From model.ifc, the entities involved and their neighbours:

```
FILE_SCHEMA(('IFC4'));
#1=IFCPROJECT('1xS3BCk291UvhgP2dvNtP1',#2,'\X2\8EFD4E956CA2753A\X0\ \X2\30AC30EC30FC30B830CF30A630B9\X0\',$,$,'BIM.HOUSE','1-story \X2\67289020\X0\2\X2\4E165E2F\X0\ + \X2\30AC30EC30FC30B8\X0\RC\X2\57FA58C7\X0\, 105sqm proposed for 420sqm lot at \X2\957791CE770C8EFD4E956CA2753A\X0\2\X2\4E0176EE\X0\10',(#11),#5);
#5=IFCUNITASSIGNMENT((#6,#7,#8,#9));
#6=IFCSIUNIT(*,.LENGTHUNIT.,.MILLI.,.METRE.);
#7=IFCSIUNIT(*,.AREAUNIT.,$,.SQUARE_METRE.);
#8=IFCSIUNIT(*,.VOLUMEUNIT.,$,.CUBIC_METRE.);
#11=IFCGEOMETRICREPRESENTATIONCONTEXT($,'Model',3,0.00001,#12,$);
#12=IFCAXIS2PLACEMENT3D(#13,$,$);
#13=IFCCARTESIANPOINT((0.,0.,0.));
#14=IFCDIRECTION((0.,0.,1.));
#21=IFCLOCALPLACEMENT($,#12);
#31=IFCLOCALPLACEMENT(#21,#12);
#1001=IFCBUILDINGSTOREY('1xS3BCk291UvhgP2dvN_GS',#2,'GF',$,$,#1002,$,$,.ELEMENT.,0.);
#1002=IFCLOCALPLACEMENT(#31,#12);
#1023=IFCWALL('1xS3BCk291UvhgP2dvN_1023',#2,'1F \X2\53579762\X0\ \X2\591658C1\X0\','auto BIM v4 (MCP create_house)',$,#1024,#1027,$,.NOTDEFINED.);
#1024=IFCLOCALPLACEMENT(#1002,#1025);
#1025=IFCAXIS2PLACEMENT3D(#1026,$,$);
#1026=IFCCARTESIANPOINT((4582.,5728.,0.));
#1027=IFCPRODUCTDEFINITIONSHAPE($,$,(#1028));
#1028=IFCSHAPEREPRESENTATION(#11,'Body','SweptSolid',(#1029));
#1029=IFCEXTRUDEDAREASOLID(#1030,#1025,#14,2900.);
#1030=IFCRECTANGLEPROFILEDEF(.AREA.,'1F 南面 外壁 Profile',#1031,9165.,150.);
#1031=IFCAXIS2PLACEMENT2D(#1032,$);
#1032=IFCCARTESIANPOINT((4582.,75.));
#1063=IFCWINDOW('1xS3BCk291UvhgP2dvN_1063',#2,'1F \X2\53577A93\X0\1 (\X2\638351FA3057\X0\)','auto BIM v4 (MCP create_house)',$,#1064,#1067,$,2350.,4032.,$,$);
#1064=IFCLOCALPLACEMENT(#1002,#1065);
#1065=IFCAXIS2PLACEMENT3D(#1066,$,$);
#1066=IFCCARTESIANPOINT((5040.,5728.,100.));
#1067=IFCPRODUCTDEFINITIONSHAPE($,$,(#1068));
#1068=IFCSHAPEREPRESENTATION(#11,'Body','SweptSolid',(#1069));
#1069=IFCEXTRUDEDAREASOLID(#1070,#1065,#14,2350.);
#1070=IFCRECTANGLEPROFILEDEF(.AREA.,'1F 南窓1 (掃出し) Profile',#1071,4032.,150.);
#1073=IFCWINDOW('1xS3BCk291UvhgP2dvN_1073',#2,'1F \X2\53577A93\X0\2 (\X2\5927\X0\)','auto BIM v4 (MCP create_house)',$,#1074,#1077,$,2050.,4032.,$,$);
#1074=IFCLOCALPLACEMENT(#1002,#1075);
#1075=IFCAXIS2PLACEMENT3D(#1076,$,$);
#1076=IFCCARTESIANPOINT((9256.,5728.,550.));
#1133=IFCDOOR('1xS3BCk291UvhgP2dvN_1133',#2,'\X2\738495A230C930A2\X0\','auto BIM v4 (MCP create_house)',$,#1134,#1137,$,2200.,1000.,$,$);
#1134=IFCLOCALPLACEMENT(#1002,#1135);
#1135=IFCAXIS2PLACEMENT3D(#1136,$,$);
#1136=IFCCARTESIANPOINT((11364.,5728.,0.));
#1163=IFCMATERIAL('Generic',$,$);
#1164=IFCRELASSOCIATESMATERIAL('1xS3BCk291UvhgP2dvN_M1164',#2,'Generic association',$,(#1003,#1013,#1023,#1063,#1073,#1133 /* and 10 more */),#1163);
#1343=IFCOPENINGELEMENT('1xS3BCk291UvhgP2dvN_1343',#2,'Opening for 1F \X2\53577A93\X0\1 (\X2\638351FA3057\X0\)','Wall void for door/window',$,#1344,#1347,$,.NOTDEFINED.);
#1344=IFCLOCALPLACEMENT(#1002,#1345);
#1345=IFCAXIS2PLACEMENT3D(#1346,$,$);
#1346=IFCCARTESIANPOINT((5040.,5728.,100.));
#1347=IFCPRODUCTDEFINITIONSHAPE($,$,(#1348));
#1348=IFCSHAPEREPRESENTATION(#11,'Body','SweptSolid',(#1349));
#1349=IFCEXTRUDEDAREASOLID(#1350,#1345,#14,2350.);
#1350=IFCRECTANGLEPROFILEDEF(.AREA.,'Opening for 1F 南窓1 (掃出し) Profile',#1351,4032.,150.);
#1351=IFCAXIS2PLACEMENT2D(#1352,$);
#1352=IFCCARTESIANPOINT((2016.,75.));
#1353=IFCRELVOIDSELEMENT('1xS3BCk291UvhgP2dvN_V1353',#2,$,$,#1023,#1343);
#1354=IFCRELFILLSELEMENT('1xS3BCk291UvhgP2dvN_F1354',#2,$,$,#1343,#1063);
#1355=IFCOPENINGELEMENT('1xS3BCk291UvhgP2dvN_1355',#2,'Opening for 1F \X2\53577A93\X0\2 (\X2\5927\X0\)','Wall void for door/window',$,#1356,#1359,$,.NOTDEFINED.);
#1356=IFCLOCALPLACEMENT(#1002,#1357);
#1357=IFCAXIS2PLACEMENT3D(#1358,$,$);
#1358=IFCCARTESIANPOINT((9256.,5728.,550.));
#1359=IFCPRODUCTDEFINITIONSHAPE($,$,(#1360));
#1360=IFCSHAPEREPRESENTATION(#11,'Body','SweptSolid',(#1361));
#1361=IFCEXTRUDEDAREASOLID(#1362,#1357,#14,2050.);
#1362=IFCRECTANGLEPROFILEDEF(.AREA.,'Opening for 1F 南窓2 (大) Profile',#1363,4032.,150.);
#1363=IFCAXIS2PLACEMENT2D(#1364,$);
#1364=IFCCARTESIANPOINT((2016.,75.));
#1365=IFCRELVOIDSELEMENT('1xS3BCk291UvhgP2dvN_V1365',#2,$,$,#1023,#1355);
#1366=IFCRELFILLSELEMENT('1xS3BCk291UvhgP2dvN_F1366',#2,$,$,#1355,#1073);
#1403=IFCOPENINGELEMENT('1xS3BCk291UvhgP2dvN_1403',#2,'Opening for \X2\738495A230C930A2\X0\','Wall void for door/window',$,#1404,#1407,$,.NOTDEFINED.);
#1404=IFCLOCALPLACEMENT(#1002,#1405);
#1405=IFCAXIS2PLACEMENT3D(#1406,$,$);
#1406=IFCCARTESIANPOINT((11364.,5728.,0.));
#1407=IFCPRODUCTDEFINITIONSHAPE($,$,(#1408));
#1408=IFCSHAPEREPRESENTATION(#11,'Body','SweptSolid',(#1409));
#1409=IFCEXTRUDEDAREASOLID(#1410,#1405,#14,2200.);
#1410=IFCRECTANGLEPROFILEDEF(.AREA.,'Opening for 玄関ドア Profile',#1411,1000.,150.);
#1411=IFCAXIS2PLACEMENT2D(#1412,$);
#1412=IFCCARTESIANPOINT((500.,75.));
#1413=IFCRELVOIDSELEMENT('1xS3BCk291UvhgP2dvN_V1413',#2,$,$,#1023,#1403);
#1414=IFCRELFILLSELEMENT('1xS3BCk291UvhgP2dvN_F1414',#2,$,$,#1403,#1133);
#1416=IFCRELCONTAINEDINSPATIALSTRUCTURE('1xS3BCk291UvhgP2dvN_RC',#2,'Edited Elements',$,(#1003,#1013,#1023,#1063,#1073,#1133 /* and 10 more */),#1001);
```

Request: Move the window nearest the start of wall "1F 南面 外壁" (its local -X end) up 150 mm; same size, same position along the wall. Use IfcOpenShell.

```python
import numpy as np
import ifcopenshell
import ifcopenshell.api.geometry
import ifcopenshell.util.placement
import ifcopenshell.util.unit

model = ifcopenshell.open("model.ifc")
unit_scale = ifcopenshell.util.unit.calculate_unit_scale(model)

window = model.by_guid("1xS3BCk291UvhgP2dvN_1063")
opening = window.FillsVoids[0].RelatingOpeningElement
dz = 150.0

shift = np.array([0.0, 0.0, dz])
# The window is not placed relative to its opening, so move both.
for product in (opening, window):
    matrix = ifcopenshell.util.placement.get_local_placement(product.ObjectPlacement)
    matrix[:3, 3] += shift
    ifcopenshell.api.geometry.edit_object_placement(model, product=product, matrix=matrix, is_si=False)

print(f"moved by {dz * unit_scale:+.3f} m")

model.write("model_v2.ifc")
```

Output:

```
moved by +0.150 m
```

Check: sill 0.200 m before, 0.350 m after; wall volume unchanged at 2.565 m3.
